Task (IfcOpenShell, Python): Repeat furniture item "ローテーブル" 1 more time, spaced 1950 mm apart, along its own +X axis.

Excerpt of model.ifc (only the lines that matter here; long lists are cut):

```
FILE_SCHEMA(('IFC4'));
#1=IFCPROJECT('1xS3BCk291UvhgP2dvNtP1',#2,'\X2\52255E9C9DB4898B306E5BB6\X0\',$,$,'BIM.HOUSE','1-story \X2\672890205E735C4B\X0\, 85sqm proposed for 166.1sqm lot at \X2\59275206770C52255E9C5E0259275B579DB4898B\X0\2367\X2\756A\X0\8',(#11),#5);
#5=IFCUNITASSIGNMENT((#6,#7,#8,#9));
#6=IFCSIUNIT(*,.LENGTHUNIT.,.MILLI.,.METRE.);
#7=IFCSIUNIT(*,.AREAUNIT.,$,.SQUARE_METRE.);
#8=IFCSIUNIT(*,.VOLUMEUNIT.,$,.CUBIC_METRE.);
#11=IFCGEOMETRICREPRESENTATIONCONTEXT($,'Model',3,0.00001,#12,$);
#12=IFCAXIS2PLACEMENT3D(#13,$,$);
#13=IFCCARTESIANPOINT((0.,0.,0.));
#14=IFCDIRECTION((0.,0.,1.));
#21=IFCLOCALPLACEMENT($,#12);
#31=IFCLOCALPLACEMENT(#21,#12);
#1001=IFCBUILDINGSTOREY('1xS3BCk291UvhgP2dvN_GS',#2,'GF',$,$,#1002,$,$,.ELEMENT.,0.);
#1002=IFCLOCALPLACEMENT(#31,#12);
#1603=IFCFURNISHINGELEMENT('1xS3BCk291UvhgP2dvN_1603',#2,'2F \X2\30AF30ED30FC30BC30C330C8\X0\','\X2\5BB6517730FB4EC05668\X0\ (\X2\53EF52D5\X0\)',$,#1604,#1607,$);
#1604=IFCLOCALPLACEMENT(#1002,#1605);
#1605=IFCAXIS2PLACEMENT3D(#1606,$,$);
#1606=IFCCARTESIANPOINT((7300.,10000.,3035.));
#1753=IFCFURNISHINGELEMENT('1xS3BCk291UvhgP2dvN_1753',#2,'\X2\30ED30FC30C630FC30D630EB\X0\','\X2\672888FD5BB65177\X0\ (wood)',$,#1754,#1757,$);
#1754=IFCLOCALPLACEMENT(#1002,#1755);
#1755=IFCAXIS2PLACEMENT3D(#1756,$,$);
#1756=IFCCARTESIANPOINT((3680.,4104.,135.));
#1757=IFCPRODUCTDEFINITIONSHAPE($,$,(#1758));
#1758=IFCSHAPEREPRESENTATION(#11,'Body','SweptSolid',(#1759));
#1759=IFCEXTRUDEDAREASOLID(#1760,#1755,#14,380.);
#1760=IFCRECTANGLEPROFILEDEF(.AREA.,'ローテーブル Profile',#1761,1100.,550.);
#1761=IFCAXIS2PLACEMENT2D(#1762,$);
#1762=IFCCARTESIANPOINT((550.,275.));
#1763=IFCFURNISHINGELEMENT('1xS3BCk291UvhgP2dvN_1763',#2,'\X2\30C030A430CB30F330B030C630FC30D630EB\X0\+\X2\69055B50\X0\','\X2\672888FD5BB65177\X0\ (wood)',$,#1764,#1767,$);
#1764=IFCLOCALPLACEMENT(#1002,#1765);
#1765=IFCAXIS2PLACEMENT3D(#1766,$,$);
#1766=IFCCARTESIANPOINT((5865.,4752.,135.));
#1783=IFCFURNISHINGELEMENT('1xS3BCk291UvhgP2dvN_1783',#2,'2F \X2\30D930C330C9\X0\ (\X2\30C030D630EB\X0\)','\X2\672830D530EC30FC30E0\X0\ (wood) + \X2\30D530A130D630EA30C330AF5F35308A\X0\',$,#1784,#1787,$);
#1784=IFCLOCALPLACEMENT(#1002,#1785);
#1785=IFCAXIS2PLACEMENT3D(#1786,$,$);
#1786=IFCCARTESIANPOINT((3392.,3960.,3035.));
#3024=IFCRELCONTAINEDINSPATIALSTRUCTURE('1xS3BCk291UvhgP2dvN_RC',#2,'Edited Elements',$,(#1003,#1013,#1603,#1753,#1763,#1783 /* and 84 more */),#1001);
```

```python
import ifcopenshell
import ifcopenshell.api.geometry
import ifcopenshell.api.root
import ifcopenshell.util.element
import ifcopenshell.util.placement
import ifcopenshell.util.unit

model = ifcopenshell.open("model.ifc")
unit_scale = ifcopenshell.util.unit.calculate_unit_scale(model)


def reuse_history(source, copy):
    """copy_class also copies each property set's owner history, people and application; keep the originals."""
    for rel in copy.IsDefinedBy:
        if rel.is_a("IfcRelDefinesByProperties") and (history := rel.RelatingPropertyDefinition.OwnerHistory):
            rel.RelatingPropertyDefinition.OwnerHistory = source.OwnerHistory
            ifcopenshell.util.element.remove_deep2(model, history)


source = model.by_guid("1xS3BCk291UvhgP2dvN_1753")
base = ifcopenshell.util.placement.get_local_placement(source.ObjectPlacement)
step = base[:3, 0] * 1.95 / unit_scale

for i in range(1, 2):
    copy = ifcopenshell.api.root.copy_class(model, product=source)
    copy.Representation = ifcopenshell.util.element.copy_deep(
        model, source.Representation, exclude=["IfcGeometricRepresentationContext", "IfcRepresentationMap"]
    )
    reuse_history(source, copy)
    matrix = base.copy()
    matrix[:3, 3] += i * step
    print("added at", matrix[:3, 3].round(3) + 0.0)
    ifcopenshell.api.geometry.edit_object_placement(model, product=copy, matrix=matrix, is_si=False)

model.write("model_updated.ifc")
```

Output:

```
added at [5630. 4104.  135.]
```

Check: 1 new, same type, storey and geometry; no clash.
